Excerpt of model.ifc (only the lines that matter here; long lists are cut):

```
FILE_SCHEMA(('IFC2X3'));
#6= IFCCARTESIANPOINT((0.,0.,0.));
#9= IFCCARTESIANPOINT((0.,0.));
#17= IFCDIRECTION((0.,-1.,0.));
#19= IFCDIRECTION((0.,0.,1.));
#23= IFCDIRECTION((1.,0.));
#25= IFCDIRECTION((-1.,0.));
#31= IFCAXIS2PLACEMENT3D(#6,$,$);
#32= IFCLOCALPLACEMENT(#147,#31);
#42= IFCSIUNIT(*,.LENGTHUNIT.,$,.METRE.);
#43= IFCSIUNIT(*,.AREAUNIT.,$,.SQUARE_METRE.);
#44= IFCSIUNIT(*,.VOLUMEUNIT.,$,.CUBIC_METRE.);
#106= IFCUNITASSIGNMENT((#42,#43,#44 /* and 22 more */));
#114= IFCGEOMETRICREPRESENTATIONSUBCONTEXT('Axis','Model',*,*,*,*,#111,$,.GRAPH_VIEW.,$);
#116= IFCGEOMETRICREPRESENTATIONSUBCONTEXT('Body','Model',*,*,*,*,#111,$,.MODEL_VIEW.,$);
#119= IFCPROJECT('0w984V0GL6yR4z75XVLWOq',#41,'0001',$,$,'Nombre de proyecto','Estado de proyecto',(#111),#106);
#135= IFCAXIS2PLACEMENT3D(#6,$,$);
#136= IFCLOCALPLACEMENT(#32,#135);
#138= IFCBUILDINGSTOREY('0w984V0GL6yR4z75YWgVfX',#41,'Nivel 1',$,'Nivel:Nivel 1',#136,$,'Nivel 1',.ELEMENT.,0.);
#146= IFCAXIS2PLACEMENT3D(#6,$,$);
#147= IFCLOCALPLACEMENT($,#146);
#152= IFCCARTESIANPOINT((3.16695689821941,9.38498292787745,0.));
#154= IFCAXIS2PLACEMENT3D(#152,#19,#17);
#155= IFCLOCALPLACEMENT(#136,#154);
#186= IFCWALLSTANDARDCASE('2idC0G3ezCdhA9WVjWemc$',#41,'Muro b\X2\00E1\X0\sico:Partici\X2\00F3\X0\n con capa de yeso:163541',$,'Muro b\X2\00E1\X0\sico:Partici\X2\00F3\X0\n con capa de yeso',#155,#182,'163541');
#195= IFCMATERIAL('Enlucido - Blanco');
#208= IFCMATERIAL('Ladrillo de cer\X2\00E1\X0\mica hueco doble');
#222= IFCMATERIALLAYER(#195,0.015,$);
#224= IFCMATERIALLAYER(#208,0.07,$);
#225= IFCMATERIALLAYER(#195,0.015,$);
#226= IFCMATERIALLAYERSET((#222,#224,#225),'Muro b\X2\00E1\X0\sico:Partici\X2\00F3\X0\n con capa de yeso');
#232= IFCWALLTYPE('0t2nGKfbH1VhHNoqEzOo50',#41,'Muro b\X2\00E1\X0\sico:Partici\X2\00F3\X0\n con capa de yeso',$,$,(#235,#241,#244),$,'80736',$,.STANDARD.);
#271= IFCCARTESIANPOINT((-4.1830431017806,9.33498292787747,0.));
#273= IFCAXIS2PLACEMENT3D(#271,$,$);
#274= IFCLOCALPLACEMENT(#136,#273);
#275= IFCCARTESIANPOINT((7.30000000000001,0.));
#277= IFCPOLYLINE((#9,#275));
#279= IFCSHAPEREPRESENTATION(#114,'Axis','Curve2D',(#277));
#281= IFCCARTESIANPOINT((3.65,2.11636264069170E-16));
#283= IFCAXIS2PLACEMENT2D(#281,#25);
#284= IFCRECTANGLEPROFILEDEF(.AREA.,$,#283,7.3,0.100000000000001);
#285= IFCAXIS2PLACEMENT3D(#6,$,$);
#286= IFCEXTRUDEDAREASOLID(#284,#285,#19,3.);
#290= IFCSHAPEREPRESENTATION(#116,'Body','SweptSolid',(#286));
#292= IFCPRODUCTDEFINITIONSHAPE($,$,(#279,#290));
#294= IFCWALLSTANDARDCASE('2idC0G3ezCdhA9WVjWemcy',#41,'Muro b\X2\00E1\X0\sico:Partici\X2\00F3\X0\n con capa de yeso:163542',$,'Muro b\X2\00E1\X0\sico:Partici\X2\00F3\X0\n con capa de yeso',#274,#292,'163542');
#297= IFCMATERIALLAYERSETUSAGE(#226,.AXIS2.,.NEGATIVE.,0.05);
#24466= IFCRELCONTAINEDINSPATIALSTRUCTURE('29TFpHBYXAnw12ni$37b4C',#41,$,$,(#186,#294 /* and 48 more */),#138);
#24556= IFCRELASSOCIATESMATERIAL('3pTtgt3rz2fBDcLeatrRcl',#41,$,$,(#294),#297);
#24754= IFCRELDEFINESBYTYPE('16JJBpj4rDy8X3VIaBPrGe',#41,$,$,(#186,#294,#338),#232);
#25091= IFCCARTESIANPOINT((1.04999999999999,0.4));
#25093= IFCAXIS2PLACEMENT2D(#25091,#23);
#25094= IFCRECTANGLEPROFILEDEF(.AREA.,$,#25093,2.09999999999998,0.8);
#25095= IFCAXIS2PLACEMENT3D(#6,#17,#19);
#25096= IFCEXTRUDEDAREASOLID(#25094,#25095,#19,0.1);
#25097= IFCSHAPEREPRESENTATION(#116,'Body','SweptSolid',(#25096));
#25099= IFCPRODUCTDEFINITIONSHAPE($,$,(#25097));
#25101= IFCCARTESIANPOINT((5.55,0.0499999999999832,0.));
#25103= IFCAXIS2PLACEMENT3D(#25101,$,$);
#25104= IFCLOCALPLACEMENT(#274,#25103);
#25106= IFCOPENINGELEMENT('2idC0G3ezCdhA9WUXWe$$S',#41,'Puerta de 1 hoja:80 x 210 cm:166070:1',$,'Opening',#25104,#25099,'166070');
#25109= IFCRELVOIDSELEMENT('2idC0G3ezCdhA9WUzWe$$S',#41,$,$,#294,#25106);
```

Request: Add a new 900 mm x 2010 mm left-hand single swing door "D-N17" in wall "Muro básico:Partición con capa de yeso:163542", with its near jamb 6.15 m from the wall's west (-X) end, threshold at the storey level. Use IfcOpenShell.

```python
import numpy as np
import ifcopenshell
import ifcopenshell.api.feature
import ifcopenshell.api.geometry
import ifcopenshell.api.root
import ifcopenshell.api.spatial
import ifcopenshell.api.type
import ifcopenshell.geom
import ifcopenshell.util.element
import ifcopenshell.util.placement
import ifcopenshell.util.representation
import ifcopenshell.util.shape
import ifcopenshell.util.unit

model = ifcopenshell.open("model.ifc")
unit_scale = ifcopenshell.util.unit.calculate_unit_scale(model)
settings = ifcopenshell.geom.settings()


def volume(element):
    """Net volume in cubic metres, openings subtracted."""
    shape = ifcopenshell.geom.create_shape(settings, element)
    return ifcopenshell.util.shape.get_volume(shape.geometry)


wall = model.by_guid("2idC0G3ezCdhA9WVjWemcy")
storey = ifcopenshell.util.element.get_container(wall, ifc_class="IfcBuildingStorey")
context = ifcopenshell.util.representation.get_context(model, "Model", "Body", "MODEL_VIEW")
before = volume(wall)

width, height, from_end, sill = 0.9, 2.01, 6.15, 0.0  # metres

# The wall runs along its own X axis, and the end named is its -X end.
wall_shape = ifcopenshell.geom.create_shape(settings, wall)
x, y, z = ifcopenshell.util.shape.get_vertices(wall_shape.geometry).T
start = x.min() + from_end
face, thickness = float(y.min()), float(y.max() - y.min())
wall_matrix = ifcopenshell.util.placement.get_local_placement(wall.ObjectPlacement)
level = ifcopenshell.util.placement.get_local_placement(storey.ObjectPlacement)[2, 3]


def in_wall(x, y):
    """Placement at x, y metres in the wall's axes, at sill height."""
    matrix = wall_matrix.copy()
    matrix[:, 3] = wall_matrix @ np.array([x / unit_scale, y / unit_scale, 0.0, 1.0])
    matrix[2, 3] = level + sill / unit_scale
    return matrix


# Opening: a box that overshoots both wall faces by 50 mm.
opening = ifcopenshell.api.root.create_entity(model, ifc_class="IfcOpeningElement")
box = ifcopenshell.api.geometry.add_wall_representation(
    model, context=context, length=width, height=height, thickness=thickness + 0.1
)
ifcopenshell.api.geometry.assign_representation(model, product=opening, representation=box)
ifcopenshell.api.geometry.edit_object_placement(model, product=opening, matrix=in_wall(start, face - 0.05), is_si=False)
ifcopenshell.api.feature.add_feature(model, feature=opening, element=wall)

door = ifcopenshell.api.root.create_entity(model, ifc_class="IfcDoor", name="D-N17")
door.OverallWidth, door.OverallHeight = width / unit_scale, height / unit_scale
body = ifcopenshell.api.geometry.add_door_representation(
    model,
    context=context,
    overall_width=door.OverallWidth,
    overall_height=door.OverallHeight,
    operation_type="SINGLE_SWING_LEFT",
    lining_properties={"LiningDepth": thickness / unit_scale, "ThresholdDepth": thickness / unit_scale},
)
ifcopenshell.api.geometry.assign_representation(model, product=door, representation=body)
ifcopenshell.api.spatial.assign_container(model, products=[door], relating_structure=storey)
fills = ifcopenshell.api.feature.add_filling(model, opening=opening, element=door)
fills.OwnerHistory = door.OwnerHistory  # required in IFC2X3

# IFC2X3 keeps the operation on the door style.
style = ifcopenshell.api.root.create_entity(model, ifc_class="IfcDoorStyle", name="D-N17")
style.OperationType, style.ConstructionType = "SINGLE_SWING_LEFT", "NOTDEFINED"
style.ParameterTakesPrecedence = style.Sizeable = False
ifcopenshell.api.type.assign_type(model, related_objects=[door], relating_type=style)

# The lining spans the wall, so the door starts at the wall face.
ifcopenshell.api.geometry.edit_object_placement(model, product=door, matrix=in_wall(start, face), is_si=False)

after = volume(wall)

print(f"wall volume {before:.3f} -> {after:.3f} m3")

model.write("model_updated.ifc")
```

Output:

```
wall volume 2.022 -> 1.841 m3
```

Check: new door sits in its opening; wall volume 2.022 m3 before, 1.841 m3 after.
